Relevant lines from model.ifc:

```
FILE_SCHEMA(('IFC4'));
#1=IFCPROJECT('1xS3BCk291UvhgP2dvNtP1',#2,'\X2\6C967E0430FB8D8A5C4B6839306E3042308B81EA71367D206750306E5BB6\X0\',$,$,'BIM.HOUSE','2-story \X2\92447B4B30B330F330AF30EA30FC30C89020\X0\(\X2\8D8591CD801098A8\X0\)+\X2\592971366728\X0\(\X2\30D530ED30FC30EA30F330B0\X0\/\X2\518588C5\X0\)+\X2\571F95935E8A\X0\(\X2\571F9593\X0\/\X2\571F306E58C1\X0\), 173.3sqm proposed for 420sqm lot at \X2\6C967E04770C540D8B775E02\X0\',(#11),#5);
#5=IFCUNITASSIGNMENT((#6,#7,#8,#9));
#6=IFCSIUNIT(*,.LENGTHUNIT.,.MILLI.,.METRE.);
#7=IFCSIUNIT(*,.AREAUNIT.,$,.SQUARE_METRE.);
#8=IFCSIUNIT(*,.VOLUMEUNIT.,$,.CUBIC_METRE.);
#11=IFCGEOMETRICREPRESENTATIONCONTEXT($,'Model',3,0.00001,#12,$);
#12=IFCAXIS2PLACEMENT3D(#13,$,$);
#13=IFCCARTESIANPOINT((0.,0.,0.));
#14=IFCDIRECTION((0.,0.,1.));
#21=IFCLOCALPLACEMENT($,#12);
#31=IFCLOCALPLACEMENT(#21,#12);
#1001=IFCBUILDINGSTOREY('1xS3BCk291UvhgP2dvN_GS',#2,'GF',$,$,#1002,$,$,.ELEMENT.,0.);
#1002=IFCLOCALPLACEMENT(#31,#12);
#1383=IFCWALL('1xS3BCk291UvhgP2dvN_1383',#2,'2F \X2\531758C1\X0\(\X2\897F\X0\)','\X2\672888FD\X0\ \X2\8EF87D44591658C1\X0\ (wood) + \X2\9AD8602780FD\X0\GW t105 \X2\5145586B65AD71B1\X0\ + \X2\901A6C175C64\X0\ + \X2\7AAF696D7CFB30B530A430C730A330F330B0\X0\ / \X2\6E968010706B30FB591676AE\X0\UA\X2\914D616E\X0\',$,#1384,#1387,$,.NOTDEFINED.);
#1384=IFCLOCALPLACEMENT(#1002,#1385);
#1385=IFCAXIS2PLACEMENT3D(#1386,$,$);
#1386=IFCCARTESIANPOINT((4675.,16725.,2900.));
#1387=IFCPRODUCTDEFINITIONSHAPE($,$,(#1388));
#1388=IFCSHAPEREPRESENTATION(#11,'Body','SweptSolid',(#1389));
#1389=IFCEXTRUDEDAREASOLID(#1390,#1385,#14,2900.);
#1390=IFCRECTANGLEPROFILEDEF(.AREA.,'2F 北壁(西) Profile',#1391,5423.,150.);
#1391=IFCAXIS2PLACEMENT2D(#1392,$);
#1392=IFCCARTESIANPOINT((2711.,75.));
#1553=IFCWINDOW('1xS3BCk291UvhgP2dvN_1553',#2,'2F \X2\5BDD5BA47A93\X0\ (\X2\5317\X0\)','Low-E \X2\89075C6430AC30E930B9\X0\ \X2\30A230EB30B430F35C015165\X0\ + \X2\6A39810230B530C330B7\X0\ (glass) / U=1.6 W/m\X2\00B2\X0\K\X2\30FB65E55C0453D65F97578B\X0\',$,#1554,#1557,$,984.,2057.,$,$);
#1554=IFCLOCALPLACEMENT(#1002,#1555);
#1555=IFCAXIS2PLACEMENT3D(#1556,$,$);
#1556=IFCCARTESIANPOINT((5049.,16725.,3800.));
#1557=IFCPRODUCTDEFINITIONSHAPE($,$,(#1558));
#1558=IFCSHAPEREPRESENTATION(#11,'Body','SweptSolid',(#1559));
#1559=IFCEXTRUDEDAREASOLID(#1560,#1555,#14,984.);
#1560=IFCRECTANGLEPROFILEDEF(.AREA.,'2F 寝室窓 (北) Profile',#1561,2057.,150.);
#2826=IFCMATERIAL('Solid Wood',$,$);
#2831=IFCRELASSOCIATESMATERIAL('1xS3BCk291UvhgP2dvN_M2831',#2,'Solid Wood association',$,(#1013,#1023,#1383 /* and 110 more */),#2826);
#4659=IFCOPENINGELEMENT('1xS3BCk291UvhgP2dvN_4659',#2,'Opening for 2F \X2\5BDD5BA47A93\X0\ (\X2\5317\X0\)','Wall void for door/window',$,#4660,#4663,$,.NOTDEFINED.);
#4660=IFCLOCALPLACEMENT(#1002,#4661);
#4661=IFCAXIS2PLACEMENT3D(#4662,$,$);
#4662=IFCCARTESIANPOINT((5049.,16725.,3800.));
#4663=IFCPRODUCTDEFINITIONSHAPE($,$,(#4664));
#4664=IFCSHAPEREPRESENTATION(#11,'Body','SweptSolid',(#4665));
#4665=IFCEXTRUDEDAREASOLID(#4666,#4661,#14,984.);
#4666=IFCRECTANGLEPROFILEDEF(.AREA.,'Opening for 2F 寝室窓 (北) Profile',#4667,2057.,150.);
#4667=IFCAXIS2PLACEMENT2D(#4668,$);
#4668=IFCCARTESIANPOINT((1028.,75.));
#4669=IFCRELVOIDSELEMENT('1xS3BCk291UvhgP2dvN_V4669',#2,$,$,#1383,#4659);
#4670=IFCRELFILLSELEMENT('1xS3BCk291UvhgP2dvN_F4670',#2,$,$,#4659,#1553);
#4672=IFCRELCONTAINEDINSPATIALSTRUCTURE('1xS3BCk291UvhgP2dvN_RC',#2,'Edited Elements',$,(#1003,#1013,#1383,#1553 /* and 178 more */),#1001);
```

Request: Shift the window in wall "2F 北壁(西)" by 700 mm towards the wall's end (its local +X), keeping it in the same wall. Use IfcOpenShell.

```python
import ifcopenshell
import ifcopenshell.api.geometry
import ifcopenshell.util.placement

model = ifcopenshell.open("model.ifc")

window = model.by_guid("1xS3BCk291UvhgP2dvN_1553")
opening = window.FillsVoids[0].RelatingOpeningElement
wall = opening.VoidsElements[0].RelatingBuildingElement

wall_matrix = ifcopenshell.util.placement.get_local_placement(wall.ObjectPlacement)
shift = wall_matrix[:3, 0] * 700.0
before = ifcopenshell.util.placement.get_local_placement(window.ObjectPlacement)[:3, 3].copy()

# The window is not placed relative to its opening, so move both.
for product in (opening, window):
    matrix = ifcopenshell.util.placement.get_local_placement(product.ObjectPlacement)
    matrix[:3, 3] += shift
    ifcopenshell.api.geometry.edit_object_placement(model, product=product, matrix=matrix, is_si=False)

after = ifcopenshell.util.placement.get_local_placement(window.ObjectPlacement)[:3, 3]
print("window moved by", (after - before).round(3) + 0.0)

model.write("model-out.ifc")
```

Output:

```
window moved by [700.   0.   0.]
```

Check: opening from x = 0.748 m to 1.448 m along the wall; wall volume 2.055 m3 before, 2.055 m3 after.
